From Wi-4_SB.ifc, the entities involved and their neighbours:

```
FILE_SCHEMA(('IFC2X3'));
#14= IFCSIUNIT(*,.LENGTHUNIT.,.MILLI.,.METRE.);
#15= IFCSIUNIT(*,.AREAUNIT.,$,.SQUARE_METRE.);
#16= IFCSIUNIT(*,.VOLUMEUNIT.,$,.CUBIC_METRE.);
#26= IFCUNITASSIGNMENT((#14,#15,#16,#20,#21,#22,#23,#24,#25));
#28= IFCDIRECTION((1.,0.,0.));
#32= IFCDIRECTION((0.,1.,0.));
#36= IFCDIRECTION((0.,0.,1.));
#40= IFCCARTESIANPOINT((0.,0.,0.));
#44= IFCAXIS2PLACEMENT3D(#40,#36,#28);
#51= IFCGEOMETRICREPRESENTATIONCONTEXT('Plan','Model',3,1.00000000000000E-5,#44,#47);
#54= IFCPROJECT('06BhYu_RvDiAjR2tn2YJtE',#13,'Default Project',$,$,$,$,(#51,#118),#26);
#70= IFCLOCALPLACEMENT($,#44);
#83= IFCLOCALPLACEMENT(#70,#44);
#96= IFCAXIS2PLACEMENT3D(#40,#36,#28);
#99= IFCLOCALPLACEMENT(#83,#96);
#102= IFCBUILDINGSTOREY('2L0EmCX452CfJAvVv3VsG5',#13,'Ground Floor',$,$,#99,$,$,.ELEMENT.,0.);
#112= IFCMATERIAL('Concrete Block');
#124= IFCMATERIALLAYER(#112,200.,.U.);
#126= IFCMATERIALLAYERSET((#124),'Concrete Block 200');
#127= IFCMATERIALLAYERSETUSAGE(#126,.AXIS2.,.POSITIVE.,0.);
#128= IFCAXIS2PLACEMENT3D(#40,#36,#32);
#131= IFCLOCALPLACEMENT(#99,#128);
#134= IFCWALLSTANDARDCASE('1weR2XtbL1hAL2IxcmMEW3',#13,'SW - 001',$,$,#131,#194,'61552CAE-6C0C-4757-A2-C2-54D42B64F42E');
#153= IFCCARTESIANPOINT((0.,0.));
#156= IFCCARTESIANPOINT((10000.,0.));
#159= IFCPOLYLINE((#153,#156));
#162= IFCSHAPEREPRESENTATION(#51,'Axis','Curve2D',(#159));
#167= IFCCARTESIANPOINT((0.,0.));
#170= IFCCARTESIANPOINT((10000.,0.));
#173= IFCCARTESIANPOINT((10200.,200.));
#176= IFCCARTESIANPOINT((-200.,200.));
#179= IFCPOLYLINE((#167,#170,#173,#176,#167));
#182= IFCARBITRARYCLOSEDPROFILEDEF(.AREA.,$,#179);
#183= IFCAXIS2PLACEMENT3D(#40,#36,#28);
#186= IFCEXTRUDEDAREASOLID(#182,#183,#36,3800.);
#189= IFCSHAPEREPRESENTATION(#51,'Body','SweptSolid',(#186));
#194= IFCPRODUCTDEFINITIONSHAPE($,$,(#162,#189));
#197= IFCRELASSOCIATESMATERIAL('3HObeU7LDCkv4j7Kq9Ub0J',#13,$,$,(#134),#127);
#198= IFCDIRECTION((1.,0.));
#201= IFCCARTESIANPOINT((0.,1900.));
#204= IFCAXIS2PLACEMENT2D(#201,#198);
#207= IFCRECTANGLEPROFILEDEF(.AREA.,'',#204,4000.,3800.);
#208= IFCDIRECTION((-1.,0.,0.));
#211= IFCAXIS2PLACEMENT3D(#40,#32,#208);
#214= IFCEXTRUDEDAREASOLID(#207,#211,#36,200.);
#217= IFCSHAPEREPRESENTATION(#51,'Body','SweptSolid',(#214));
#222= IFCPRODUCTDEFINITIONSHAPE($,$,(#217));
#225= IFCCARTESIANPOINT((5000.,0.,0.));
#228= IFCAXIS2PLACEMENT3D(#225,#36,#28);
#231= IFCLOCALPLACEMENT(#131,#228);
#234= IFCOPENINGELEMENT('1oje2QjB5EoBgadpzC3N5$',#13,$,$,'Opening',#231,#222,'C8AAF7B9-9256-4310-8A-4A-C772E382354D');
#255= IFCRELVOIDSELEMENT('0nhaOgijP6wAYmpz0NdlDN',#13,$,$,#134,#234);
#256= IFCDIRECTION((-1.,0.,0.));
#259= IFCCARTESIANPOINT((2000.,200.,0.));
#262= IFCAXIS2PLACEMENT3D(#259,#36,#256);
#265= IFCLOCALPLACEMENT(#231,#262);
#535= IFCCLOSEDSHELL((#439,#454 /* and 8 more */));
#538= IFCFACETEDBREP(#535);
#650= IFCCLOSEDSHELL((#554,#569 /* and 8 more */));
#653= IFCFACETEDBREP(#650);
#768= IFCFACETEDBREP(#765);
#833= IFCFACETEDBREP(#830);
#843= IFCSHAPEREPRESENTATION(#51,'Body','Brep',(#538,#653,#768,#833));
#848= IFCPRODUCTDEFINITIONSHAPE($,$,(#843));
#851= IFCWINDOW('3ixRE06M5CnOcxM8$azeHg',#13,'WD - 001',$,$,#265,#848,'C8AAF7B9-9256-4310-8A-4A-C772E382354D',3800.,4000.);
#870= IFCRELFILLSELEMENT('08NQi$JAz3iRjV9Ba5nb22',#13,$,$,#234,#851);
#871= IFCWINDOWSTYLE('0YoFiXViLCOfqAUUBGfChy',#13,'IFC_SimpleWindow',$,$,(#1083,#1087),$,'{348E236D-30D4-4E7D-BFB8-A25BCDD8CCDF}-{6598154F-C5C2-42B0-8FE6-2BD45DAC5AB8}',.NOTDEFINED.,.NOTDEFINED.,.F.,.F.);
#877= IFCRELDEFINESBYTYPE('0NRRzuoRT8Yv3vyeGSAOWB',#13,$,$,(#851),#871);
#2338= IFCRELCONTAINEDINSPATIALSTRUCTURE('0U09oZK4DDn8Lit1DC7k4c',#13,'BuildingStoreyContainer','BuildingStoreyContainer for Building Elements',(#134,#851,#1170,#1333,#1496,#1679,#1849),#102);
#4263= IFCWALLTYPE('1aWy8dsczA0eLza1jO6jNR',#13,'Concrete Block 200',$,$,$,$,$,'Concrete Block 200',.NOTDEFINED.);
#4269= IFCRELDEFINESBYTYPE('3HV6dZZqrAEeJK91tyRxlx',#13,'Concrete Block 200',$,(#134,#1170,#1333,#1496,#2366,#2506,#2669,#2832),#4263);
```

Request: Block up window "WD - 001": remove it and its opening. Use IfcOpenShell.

```python
import ifcopenshell
import ifcopenshell.api.feature
import ifcopenshell.api.root
import ifcopenshell.geom
import ifcopenshell.util.shape

model = ifcopenshell.open("Wi-4_SB.ifc")
settings = ifcopenshell.geom.settings()


def volume(element):
    """Net volume in cubic metres, openings subtracted."""
    shape = ifcopenshell.geom.create_shape(settings, element)
    return ifcopenshell.util.shape.get_volume(shape.geometry)


window = model.by_id(851)
opening = window.FillsVoids[0].RelatingOpeningElement
wall = opening.VoidsElements[0].RelatingBuildingElement
before = volume(wall)

ifcopenshell.api.root.remove_product(model, product=window)
ifcopenshell.api.feature.remove_feature(model, feature=opening)

after = volume(wall)

print(f"wall volume {before:.3f} -> {after:.3f} m3")

model.write("Wi-4_SB_rev.ifc")
```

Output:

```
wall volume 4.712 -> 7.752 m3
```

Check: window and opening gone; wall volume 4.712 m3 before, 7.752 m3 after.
